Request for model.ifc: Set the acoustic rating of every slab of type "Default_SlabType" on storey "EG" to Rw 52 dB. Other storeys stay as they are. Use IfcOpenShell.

First a look at what the model holds.

```python
import ifcopenshell
import ifcopenshell.util.element

model = ifcopenshell.open("model.ifc")
print(model.schema)
storey = next(s for s in model.by_type("IfcBuildingStorey") if s.Name == "EG")
slabs = [e for e in ifcopenshell.util.element.get_decomposition(storey) if e.is_a("IfcSlab")]
seen = {}
for e in slabs:
    element_type = ifcopenshell.util.element.get_type(e)
    key = (element_type.Name if element_type != e and element_type else None, ifcopenshell.util.element.get_pset(e, "Pset_SlabCommon", "AcousticRating"))
    seen[key] = seen.get(key, 0) + 1
for (name, value), count in sorted(seen.items(), key=str):
    print(count, "x", name, "|", value)
```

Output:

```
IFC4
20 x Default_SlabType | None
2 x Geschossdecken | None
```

```python
import ifcopenshell
import ifcopenshell.api.pset
import ifcopenshell.util.element

model = ifcopenshell.open("model.ifc")

storey = next(s for s in model.by_type("IfcBuildingStorey") if s.Name == "EG")
slabs = [e for e in ifcopenshell.util.element.get_decomposition(storey) if e.is_a("IfcSlab")]

count = 0
for e in slabs:
    element_type = ifcopenshell.util.element.get_type(e)
    if element_type in (None, e) or element_type.Name != "Default_SlabType":
        continue
    # add_pset returns the element's existing set when there is one.
    pset = ifcopenshell.api.pset.add_pset(model, product=e, name="Pset_SlabCommon")
    ifcopenshell.api.pset.edit_pset(model, pset=pset, properties={"AcousticRating": "Rw 52 dB"})
    count += 1

print(count, "slabs updated")

model.write("model_rev.ifc")
```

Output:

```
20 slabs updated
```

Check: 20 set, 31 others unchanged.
